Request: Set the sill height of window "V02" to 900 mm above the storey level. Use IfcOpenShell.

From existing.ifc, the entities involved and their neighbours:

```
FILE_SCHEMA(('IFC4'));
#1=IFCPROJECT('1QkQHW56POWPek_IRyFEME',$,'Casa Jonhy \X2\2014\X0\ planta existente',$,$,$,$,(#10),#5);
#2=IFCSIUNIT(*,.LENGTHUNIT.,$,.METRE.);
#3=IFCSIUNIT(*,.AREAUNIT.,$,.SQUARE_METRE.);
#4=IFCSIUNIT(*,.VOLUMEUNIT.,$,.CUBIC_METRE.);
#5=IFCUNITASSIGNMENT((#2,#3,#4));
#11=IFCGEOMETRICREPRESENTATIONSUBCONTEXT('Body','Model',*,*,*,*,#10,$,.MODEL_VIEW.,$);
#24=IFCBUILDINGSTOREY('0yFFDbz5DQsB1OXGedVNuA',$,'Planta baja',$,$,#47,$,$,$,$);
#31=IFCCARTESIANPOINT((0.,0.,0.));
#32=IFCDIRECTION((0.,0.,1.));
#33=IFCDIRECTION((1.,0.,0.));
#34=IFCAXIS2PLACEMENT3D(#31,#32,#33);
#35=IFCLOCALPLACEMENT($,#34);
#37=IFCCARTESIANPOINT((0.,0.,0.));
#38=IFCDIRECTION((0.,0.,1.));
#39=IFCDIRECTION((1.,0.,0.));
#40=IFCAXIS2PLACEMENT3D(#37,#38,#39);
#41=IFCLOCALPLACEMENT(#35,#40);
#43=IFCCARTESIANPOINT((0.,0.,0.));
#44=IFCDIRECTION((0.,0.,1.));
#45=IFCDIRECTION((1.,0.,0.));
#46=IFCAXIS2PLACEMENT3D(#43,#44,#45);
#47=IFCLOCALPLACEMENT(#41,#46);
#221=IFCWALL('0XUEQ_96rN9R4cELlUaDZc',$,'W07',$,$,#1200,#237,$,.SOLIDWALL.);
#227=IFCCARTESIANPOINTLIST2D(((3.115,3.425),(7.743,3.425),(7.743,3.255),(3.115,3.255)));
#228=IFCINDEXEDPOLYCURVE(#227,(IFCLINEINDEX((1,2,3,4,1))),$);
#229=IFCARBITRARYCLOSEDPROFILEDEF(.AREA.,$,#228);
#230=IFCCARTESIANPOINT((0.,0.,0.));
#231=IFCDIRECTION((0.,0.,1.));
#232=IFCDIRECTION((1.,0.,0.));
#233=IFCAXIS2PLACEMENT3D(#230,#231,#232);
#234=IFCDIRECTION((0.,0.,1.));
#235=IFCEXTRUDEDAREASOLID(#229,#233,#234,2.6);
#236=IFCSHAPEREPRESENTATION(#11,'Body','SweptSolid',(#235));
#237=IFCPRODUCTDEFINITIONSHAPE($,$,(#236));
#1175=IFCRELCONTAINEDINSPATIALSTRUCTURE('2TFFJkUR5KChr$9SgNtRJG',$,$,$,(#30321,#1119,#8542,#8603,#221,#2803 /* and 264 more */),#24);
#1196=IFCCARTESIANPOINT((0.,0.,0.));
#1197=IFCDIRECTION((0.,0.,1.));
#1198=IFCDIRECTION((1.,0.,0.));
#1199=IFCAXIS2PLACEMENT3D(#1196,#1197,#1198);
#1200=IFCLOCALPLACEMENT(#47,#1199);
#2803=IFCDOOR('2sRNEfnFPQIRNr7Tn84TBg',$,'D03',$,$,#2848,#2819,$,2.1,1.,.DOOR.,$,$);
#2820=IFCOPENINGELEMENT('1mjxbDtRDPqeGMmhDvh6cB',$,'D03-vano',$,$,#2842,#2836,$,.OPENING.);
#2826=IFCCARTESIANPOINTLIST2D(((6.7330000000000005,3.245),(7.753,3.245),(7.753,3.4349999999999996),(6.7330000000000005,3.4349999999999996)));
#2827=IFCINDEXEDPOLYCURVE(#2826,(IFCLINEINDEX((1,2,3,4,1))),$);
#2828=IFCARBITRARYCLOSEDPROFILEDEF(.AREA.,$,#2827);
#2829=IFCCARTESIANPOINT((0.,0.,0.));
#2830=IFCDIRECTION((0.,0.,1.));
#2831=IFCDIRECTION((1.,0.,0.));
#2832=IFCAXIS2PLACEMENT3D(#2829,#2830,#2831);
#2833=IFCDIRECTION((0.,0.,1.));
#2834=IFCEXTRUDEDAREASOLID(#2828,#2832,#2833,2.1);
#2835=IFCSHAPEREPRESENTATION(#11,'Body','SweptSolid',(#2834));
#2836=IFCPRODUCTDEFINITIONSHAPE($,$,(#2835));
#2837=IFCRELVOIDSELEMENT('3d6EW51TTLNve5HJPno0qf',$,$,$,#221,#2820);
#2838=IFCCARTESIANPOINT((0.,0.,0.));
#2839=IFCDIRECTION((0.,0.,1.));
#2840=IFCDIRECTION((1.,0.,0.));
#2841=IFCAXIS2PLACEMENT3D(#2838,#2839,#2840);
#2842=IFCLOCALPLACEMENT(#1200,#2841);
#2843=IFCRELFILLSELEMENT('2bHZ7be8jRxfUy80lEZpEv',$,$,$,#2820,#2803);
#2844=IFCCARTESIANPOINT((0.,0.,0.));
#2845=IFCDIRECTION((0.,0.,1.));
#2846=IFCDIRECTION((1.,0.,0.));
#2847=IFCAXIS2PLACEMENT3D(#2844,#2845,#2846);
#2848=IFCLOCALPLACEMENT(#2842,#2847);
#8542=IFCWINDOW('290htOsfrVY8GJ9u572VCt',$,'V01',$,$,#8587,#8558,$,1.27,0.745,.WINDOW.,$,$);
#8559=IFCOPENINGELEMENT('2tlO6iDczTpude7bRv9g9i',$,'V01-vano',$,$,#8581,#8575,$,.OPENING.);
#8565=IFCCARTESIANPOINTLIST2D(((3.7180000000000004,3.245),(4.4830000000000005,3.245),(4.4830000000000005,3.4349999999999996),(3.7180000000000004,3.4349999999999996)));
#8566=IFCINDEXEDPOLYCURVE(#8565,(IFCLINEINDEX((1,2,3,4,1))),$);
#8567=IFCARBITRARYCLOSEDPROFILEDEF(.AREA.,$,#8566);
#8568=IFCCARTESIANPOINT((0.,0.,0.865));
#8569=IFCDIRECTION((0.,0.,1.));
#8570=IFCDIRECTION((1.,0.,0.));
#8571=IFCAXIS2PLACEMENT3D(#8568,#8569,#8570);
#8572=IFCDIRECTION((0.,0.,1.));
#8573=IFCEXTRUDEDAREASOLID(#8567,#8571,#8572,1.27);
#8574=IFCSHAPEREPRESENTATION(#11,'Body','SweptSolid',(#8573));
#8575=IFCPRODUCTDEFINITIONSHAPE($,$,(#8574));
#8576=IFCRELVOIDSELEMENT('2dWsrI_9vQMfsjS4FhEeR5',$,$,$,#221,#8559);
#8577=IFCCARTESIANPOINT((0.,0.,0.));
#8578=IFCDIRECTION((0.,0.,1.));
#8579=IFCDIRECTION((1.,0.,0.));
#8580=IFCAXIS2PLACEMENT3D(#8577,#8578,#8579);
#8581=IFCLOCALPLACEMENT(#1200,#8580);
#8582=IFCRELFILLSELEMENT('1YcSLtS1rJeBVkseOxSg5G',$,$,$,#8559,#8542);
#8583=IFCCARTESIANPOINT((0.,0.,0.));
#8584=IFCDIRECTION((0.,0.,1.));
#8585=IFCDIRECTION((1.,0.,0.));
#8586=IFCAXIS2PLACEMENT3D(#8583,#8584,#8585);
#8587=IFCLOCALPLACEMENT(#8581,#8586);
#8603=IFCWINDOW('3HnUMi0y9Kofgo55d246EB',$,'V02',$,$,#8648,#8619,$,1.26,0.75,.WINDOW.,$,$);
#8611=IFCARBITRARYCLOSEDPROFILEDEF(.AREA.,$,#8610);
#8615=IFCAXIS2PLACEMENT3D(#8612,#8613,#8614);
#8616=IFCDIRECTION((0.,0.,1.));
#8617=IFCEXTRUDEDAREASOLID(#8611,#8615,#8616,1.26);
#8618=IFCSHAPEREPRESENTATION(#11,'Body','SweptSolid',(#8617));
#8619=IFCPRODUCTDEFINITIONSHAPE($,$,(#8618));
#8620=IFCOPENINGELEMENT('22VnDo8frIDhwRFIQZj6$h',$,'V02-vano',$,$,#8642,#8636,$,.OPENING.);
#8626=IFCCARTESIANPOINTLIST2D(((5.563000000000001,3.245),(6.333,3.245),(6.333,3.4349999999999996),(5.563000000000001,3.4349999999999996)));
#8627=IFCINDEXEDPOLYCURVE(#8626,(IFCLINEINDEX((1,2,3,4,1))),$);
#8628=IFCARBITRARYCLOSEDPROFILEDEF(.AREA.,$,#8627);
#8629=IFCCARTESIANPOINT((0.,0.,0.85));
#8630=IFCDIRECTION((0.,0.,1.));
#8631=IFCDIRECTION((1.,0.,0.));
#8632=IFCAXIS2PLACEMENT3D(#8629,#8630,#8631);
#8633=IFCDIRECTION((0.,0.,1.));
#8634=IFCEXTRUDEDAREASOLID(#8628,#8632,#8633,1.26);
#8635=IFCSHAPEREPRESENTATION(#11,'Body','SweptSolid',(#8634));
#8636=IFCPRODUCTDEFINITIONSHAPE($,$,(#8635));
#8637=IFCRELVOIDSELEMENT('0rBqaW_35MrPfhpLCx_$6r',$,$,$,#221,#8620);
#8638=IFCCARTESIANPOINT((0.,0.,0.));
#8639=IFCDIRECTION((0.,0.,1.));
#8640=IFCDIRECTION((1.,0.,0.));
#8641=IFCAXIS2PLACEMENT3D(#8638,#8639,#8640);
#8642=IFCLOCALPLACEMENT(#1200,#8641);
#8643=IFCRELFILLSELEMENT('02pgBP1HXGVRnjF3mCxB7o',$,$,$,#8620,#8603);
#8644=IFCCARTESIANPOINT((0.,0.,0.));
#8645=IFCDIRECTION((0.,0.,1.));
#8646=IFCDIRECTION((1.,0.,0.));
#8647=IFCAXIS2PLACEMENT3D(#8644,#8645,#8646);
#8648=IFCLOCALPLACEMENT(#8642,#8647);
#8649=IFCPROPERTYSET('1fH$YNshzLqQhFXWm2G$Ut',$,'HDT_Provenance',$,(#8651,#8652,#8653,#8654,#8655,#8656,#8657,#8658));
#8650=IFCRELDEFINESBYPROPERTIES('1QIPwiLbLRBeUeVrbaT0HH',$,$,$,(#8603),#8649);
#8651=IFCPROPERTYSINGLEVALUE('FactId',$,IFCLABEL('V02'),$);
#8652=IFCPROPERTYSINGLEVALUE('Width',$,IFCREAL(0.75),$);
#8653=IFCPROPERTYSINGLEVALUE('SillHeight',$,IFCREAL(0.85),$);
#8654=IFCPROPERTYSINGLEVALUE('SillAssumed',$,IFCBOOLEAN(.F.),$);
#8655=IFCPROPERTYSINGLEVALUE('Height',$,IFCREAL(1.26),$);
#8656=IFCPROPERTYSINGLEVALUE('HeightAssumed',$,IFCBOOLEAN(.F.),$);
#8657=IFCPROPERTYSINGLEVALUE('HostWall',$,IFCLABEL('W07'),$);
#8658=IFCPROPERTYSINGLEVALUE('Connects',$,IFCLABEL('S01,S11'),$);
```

```python
import numpy as np
import ifcopenshell
import ifcopenshell.api.geometry
import ifcopenshell.api.pset
import ifcopenshell.geom
import ifcopenshell.util.element
import ifcopenshell.util.placement
import ifcopenshell.util.shape
import ifcopenshell.util.unit

model = ifcopenshell.open("existing.ifc")
unit_scale = ifcopenshell.util.unit.calculate_unit_scale(model)

window = model.by_guid("3HnUMi0y9Kofgo55d246EB")
opening = window.FillsVoids[0].RelatingOpeningElement
storey = ifcopenshell.util.element.get_container(window, ifc_class="IfcBuildingStorey")
level = ifcopenshell.util.placement.get_local_placement(storey.ObjectPlacement)[2, 3]

# The opening's origin need not be at the sill, so measure its lowest point.
shape = ifcopenshell.geom.create_shape(ifcopenshell.geom.settings(), opening)
bottom = ifcopenshell.util.shape.get_shape_bottom_elevation(shape, shape.geometry) / unit_scale
dz = level + 0.9 / unit_scale - bottom

shift = np.array([0.0, 0.0, dz])
# The window is placed relative to its opening, so it follows when the opening moves.
matrix = ifcopenshell.util.placement.get_local_placement(opening.ObjectPlacement)
matrix[:3, 3] += shift
ifcopenshell.api.geometry.edit_object_placement(
    model, product=opening, matrix=matrix, is_si=False, should_transform_children=True
)

# Keep the stored heights in step.
pset = model.by_id(ifcopenshell.util.element.get_pset(window, "HDT_Provenance", should_inherit=False)["id"])
ifcopenshell.api.pset.edit_pset(model, pset=pset, properties={
    "SillHeight": model.create_entity("IfcReal", ifcopenshell.util.element.get_pset(window, "HDT_Provenance", "SillHeight") + dz),
})

print(f"moved by {dz * unit_scale:+.3f} m")

model.write("existing_updated.ifc")
```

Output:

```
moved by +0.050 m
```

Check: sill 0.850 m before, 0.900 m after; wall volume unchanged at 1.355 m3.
